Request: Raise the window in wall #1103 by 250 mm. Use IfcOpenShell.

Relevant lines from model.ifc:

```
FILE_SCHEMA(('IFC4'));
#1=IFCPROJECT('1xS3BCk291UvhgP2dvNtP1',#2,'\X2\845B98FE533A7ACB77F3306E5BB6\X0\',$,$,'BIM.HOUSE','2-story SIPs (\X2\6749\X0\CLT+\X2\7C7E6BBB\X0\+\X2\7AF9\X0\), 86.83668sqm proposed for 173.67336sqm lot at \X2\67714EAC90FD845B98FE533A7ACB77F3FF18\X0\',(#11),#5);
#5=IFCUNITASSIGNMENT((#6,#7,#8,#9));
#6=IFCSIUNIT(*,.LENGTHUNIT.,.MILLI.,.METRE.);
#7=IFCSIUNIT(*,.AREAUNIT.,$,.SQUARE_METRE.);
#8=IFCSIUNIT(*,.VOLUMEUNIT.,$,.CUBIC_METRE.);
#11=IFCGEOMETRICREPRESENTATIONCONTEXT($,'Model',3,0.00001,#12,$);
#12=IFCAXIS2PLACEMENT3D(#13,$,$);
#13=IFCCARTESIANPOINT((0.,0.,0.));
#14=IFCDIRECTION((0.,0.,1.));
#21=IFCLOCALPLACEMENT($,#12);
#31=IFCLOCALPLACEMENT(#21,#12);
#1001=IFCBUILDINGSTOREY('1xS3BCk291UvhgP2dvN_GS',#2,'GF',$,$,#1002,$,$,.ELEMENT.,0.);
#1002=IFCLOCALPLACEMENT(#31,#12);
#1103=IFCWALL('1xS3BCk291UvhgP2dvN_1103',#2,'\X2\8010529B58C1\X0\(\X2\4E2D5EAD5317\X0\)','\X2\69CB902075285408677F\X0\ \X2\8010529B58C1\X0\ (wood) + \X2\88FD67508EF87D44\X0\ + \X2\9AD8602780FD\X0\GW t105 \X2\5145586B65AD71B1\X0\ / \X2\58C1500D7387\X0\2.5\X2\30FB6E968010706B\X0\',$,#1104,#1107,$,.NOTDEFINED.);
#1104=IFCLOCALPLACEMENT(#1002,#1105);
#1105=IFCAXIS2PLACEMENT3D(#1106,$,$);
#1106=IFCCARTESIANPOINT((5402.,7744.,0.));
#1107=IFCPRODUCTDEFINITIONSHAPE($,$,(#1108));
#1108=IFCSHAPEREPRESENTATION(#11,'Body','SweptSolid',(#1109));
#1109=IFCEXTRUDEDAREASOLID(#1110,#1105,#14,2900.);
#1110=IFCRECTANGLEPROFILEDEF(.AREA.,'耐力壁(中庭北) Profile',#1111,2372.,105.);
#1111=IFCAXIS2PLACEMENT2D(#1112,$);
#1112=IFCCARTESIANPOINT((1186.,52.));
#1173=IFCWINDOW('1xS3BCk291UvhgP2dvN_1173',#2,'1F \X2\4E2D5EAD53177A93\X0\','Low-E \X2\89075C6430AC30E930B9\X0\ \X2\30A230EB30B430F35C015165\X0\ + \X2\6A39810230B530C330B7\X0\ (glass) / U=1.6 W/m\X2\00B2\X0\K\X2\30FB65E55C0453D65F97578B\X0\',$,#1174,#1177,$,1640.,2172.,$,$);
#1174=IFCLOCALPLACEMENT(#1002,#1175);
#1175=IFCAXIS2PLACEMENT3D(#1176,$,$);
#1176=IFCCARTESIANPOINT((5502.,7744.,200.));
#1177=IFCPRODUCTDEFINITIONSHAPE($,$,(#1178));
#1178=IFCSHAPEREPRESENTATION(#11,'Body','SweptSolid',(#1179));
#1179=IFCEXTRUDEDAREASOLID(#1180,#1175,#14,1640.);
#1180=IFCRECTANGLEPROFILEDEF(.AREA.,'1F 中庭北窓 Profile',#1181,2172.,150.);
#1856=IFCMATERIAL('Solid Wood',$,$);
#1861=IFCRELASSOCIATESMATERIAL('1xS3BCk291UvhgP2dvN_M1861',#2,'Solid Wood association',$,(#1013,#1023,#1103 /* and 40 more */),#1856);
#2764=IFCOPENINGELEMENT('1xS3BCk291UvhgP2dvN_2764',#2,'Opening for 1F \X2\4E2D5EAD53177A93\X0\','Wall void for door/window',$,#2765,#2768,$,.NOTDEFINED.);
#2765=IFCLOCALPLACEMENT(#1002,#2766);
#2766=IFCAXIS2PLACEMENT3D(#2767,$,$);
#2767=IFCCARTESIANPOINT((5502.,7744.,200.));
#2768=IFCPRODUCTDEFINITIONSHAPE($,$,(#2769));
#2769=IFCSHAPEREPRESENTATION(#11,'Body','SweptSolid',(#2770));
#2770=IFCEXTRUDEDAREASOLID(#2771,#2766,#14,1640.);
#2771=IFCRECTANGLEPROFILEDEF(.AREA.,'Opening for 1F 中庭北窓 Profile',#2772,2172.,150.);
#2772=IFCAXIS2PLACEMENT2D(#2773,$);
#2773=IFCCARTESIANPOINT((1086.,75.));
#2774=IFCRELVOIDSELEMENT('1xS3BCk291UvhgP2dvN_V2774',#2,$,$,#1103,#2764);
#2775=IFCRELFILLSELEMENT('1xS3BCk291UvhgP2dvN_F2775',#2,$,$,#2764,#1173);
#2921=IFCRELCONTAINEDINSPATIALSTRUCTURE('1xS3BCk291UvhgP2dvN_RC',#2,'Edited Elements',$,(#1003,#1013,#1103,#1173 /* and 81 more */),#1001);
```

```python
import numpy as np
import ifcopenshell
import ifcopenshell.api.geometry
import ifcopenshell.util.placement
import ifcopenshell.util.unit

model = ifcopenshell.open("model.ifc")
unit_scale = ifcopenshell.util.unit.calculate_unit_scale(model)

window = model.by_id(1173)
opening = window.FillsVoids[0].RelatingOpeningElement
dz = 250.0

shift = np.array([0.0, 0.0, dz])
# The window is not placed relative to its opening, so move both.
for product in (opening, window):
    matrix = ifcopenshell.util.placement.get_local_placement(product.ObjectPlacement)
    matrix[:3, 3] += shift
    ifcopenshell.api.geometry.edit_object_placement(model, product=product, matrix=matrix, is_si=False)

print(f"moved by {dz * unit_scale:+.3f} m")

model.write("model_updated.ifc")
```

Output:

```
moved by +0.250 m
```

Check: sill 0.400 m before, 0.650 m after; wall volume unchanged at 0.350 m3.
